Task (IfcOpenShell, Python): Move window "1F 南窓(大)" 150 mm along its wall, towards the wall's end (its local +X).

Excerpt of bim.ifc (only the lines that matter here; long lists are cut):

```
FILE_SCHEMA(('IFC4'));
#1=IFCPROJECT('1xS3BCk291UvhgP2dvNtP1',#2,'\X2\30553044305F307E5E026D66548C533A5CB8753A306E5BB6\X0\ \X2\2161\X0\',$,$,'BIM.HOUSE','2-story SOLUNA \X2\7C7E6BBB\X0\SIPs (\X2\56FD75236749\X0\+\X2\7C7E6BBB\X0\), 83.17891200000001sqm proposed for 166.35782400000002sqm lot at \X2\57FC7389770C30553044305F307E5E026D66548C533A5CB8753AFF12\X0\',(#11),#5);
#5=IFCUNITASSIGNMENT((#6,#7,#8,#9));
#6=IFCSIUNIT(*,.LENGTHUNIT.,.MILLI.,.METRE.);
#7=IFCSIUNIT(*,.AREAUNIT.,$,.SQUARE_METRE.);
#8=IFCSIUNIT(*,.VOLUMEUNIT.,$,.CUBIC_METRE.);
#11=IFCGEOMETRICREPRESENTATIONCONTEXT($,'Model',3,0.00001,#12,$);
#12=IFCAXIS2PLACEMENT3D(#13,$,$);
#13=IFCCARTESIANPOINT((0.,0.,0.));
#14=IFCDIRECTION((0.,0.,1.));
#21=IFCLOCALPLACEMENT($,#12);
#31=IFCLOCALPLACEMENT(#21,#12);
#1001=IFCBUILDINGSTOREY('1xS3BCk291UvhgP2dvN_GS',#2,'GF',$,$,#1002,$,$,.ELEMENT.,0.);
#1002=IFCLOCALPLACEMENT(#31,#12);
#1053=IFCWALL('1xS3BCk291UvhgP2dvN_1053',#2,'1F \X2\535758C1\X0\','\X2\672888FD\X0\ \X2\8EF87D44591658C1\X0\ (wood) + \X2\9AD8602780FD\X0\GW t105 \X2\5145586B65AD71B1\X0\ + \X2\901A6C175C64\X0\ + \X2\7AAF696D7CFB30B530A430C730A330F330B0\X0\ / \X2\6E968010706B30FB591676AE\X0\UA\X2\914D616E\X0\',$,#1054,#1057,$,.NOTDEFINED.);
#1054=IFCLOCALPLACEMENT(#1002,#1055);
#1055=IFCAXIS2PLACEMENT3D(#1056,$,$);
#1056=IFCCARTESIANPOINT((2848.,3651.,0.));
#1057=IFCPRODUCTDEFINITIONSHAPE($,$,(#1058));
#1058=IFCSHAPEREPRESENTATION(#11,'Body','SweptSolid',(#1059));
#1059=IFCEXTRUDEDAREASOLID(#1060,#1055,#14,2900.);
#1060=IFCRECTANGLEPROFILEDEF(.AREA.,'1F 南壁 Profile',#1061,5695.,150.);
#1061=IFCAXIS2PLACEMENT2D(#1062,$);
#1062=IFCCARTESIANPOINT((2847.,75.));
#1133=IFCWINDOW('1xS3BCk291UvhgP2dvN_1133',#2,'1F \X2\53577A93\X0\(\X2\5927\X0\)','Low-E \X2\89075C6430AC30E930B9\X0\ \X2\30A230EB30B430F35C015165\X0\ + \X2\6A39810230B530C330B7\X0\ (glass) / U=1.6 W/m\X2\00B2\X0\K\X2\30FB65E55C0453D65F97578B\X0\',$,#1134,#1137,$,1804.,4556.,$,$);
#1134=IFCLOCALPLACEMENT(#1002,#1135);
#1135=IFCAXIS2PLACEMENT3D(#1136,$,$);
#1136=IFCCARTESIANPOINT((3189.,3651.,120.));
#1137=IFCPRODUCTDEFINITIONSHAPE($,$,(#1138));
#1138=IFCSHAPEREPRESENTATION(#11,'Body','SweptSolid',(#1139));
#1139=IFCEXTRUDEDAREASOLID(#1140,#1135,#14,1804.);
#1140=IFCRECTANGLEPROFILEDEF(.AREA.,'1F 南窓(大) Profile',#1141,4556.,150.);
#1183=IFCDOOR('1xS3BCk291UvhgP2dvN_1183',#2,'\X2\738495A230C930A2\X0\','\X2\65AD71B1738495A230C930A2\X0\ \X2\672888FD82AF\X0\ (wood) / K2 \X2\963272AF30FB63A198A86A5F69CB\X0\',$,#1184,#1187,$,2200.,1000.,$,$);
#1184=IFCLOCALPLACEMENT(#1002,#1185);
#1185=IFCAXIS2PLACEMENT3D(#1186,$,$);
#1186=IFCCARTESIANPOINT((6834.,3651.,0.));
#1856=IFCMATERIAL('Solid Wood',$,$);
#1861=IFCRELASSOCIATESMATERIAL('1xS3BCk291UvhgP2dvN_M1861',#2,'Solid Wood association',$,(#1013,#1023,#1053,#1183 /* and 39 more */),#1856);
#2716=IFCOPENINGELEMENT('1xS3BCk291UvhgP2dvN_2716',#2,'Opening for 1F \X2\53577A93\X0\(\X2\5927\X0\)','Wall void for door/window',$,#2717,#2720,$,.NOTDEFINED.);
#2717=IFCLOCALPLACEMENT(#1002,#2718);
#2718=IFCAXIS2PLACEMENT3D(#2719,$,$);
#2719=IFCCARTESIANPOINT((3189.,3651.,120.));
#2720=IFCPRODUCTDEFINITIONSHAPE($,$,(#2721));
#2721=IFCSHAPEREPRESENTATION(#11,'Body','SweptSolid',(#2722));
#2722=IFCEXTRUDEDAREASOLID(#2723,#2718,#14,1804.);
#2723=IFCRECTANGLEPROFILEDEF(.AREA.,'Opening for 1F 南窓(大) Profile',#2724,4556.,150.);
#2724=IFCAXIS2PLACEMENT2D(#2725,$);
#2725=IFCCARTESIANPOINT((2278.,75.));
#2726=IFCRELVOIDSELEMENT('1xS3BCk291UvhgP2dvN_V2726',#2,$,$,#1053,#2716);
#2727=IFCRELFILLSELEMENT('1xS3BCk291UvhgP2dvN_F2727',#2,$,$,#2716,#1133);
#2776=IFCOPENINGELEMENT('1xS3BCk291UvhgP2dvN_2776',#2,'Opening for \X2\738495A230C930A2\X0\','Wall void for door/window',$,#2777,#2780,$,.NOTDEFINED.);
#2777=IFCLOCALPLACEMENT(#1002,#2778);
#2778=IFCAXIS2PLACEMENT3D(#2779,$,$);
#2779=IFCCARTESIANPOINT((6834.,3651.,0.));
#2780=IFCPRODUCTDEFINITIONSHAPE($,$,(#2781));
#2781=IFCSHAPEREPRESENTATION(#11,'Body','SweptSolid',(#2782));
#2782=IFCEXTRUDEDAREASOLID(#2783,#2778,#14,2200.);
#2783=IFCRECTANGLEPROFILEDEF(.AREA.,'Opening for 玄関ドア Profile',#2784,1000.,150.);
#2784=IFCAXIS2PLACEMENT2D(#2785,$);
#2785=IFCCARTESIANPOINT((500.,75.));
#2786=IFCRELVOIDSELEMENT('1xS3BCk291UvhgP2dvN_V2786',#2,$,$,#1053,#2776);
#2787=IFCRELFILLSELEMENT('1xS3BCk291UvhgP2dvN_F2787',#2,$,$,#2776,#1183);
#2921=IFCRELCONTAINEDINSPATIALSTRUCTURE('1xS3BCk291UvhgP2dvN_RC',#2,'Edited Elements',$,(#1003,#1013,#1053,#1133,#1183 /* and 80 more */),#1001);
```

```python
import ifcopenshell
import ifcopenshell.api.geometry
import ifcopenshell.util.placement

model = ifcopenshell.open("bim.ifc")

window = model.by_guid("1xS3BCk291UvhgP2dvN_1133")
opening = window.FillsVoids[0].RelatingOpeningElement
wall = opening.VoidsElements[0].RelatingBuildingElement

wall_matrix = ifcopenshell.util.placement.get_local_placement(wall.ObjectPlacement)
shift = wall_matrix[:3, 0] * 150.0
before = ifcopenshell.util.placement.get_local_placement(window.ObjectPlacement)[:3, 3].copy()

# The window is not placed relative to its opening, so move both.
for product in (opening, window):
    matrix = ifcopenshell.util.placement.get_local_placement(product.ObjectPlacement)
    matrix[:3, 3] += shift
    ifcopenshell.api.geometry.edit_object_placement(model, product=product, matrix=matrix, is_si=False)

after = ifcopenshell.util.placement.get_local_placement(window.ObjectPlacement)[:3, 3]
print("window moved by", (after - before).round(3) + 0.0)

model.write("bim_v2.ifc")
```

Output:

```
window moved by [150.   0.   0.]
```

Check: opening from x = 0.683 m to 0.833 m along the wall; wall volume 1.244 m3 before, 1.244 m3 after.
